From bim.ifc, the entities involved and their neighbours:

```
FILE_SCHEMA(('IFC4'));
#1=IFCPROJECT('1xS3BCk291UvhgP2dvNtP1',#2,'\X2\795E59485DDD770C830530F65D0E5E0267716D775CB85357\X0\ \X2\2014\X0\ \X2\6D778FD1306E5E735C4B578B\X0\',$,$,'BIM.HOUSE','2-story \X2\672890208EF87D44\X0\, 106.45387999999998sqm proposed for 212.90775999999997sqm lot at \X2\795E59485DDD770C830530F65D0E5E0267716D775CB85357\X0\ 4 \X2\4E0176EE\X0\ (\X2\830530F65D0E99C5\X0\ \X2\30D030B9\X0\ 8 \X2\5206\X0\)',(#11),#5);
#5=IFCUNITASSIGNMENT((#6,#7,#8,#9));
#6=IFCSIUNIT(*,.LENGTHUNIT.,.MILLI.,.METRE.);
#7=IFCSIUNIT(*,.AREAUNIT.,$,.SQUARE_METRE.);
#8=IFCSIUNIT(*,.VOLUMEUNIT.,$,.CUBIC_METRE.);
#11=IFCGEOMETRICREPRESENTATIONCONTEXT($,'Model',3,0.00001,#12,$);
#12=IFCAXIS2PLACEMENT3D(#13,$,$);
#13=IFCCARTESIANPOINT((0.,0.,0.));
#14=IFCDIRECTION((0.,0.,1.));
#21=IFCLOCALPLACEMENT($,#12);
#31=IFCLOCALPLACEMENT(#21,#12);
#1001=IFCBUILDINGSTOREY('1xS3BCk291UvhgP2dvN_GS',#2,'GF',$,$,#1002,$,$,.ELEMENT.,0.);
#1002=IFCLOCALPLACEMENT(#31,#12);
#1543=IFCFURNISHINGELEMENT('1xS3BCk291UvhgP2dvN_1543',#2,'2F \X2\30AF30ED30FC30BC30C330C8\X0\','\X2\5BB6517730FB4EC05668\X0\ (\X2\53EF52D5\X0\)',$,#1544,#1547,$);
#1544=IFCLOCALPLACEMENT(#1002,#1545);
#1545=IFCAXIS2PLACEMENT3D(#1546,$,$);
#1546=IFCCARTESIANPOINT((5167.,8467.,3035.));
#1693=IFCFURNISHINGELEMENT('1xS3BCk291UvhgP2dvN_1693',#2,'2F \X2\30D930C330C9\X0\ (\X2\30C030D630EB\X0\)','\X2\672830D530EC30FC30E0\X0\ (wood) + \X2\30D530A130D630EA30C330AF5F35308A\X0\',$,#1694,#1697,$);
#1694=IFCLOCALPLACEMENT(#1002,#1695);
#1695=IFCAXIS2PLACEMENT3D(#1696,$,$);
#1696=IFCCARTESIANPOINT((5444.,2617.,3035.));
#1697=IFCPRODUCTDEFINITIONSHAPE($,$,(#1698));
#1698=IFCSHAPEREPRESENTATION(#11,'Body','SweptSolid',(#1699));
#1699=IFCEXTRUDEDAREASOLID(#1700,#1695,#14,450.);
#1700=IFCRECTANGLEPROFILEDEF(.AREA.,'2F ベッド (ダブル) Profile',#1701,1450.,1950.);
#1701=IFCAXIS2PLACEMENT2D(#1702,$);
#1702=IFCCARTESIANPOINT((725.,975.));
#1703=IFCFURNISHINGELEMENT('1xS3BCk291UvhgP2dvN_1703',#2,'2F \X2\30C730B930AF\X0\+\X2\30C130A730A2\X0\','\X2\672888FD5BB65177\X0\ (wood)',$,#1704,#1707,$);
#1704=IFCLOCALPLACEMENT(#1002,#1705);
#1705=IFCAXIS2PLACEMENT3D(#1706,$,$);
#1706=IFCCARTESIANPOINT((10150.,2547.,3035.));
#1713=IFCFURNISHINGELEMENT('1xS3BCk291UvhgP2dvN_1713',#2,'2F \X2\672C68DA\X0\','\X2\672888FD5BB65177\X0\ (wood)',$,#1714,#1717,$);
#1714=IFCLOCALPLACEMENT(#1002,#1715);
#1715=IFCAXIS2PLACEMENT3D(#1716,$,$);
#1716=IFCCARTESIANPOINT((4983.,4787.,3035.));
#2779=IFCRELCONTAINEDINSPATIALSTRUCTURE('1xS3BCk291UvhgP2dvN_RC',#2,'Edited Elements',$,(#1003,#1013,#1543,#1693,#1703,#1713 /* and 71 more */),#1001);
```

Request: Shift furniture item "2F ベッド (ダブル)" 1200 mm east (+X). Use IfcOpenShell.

```python
import ifcopenshell
import ifcopenshell.api.geometry
import ifcopenshell.util.placement

model = ifcopenshell.open("bim.ifc")

item = model.by_guid("1xS3BCk291UvhgP2dvN_1693")
matrix = ifcopenshell.util.placement.get_local_placement(item.ObjectPlacement)
matrix[0, 3] += 1200.0
ifcopenshell.api.geometry.edit_object_placement(model, product=item, matrix=matrix, is_si=False)

print(ifcopenshell.util.placement.get_local_placement(item.ObjectPlacement).round(3) + 0.0)

model.write("bim-out.ifc")
```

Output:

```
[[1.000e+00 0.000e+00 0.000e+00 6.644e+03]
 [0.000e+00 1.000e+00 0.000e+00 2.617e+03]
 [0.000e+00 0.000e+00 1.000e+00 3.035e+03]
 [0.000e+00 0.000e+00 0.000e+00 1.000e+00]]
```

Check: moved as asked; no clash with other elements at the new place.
